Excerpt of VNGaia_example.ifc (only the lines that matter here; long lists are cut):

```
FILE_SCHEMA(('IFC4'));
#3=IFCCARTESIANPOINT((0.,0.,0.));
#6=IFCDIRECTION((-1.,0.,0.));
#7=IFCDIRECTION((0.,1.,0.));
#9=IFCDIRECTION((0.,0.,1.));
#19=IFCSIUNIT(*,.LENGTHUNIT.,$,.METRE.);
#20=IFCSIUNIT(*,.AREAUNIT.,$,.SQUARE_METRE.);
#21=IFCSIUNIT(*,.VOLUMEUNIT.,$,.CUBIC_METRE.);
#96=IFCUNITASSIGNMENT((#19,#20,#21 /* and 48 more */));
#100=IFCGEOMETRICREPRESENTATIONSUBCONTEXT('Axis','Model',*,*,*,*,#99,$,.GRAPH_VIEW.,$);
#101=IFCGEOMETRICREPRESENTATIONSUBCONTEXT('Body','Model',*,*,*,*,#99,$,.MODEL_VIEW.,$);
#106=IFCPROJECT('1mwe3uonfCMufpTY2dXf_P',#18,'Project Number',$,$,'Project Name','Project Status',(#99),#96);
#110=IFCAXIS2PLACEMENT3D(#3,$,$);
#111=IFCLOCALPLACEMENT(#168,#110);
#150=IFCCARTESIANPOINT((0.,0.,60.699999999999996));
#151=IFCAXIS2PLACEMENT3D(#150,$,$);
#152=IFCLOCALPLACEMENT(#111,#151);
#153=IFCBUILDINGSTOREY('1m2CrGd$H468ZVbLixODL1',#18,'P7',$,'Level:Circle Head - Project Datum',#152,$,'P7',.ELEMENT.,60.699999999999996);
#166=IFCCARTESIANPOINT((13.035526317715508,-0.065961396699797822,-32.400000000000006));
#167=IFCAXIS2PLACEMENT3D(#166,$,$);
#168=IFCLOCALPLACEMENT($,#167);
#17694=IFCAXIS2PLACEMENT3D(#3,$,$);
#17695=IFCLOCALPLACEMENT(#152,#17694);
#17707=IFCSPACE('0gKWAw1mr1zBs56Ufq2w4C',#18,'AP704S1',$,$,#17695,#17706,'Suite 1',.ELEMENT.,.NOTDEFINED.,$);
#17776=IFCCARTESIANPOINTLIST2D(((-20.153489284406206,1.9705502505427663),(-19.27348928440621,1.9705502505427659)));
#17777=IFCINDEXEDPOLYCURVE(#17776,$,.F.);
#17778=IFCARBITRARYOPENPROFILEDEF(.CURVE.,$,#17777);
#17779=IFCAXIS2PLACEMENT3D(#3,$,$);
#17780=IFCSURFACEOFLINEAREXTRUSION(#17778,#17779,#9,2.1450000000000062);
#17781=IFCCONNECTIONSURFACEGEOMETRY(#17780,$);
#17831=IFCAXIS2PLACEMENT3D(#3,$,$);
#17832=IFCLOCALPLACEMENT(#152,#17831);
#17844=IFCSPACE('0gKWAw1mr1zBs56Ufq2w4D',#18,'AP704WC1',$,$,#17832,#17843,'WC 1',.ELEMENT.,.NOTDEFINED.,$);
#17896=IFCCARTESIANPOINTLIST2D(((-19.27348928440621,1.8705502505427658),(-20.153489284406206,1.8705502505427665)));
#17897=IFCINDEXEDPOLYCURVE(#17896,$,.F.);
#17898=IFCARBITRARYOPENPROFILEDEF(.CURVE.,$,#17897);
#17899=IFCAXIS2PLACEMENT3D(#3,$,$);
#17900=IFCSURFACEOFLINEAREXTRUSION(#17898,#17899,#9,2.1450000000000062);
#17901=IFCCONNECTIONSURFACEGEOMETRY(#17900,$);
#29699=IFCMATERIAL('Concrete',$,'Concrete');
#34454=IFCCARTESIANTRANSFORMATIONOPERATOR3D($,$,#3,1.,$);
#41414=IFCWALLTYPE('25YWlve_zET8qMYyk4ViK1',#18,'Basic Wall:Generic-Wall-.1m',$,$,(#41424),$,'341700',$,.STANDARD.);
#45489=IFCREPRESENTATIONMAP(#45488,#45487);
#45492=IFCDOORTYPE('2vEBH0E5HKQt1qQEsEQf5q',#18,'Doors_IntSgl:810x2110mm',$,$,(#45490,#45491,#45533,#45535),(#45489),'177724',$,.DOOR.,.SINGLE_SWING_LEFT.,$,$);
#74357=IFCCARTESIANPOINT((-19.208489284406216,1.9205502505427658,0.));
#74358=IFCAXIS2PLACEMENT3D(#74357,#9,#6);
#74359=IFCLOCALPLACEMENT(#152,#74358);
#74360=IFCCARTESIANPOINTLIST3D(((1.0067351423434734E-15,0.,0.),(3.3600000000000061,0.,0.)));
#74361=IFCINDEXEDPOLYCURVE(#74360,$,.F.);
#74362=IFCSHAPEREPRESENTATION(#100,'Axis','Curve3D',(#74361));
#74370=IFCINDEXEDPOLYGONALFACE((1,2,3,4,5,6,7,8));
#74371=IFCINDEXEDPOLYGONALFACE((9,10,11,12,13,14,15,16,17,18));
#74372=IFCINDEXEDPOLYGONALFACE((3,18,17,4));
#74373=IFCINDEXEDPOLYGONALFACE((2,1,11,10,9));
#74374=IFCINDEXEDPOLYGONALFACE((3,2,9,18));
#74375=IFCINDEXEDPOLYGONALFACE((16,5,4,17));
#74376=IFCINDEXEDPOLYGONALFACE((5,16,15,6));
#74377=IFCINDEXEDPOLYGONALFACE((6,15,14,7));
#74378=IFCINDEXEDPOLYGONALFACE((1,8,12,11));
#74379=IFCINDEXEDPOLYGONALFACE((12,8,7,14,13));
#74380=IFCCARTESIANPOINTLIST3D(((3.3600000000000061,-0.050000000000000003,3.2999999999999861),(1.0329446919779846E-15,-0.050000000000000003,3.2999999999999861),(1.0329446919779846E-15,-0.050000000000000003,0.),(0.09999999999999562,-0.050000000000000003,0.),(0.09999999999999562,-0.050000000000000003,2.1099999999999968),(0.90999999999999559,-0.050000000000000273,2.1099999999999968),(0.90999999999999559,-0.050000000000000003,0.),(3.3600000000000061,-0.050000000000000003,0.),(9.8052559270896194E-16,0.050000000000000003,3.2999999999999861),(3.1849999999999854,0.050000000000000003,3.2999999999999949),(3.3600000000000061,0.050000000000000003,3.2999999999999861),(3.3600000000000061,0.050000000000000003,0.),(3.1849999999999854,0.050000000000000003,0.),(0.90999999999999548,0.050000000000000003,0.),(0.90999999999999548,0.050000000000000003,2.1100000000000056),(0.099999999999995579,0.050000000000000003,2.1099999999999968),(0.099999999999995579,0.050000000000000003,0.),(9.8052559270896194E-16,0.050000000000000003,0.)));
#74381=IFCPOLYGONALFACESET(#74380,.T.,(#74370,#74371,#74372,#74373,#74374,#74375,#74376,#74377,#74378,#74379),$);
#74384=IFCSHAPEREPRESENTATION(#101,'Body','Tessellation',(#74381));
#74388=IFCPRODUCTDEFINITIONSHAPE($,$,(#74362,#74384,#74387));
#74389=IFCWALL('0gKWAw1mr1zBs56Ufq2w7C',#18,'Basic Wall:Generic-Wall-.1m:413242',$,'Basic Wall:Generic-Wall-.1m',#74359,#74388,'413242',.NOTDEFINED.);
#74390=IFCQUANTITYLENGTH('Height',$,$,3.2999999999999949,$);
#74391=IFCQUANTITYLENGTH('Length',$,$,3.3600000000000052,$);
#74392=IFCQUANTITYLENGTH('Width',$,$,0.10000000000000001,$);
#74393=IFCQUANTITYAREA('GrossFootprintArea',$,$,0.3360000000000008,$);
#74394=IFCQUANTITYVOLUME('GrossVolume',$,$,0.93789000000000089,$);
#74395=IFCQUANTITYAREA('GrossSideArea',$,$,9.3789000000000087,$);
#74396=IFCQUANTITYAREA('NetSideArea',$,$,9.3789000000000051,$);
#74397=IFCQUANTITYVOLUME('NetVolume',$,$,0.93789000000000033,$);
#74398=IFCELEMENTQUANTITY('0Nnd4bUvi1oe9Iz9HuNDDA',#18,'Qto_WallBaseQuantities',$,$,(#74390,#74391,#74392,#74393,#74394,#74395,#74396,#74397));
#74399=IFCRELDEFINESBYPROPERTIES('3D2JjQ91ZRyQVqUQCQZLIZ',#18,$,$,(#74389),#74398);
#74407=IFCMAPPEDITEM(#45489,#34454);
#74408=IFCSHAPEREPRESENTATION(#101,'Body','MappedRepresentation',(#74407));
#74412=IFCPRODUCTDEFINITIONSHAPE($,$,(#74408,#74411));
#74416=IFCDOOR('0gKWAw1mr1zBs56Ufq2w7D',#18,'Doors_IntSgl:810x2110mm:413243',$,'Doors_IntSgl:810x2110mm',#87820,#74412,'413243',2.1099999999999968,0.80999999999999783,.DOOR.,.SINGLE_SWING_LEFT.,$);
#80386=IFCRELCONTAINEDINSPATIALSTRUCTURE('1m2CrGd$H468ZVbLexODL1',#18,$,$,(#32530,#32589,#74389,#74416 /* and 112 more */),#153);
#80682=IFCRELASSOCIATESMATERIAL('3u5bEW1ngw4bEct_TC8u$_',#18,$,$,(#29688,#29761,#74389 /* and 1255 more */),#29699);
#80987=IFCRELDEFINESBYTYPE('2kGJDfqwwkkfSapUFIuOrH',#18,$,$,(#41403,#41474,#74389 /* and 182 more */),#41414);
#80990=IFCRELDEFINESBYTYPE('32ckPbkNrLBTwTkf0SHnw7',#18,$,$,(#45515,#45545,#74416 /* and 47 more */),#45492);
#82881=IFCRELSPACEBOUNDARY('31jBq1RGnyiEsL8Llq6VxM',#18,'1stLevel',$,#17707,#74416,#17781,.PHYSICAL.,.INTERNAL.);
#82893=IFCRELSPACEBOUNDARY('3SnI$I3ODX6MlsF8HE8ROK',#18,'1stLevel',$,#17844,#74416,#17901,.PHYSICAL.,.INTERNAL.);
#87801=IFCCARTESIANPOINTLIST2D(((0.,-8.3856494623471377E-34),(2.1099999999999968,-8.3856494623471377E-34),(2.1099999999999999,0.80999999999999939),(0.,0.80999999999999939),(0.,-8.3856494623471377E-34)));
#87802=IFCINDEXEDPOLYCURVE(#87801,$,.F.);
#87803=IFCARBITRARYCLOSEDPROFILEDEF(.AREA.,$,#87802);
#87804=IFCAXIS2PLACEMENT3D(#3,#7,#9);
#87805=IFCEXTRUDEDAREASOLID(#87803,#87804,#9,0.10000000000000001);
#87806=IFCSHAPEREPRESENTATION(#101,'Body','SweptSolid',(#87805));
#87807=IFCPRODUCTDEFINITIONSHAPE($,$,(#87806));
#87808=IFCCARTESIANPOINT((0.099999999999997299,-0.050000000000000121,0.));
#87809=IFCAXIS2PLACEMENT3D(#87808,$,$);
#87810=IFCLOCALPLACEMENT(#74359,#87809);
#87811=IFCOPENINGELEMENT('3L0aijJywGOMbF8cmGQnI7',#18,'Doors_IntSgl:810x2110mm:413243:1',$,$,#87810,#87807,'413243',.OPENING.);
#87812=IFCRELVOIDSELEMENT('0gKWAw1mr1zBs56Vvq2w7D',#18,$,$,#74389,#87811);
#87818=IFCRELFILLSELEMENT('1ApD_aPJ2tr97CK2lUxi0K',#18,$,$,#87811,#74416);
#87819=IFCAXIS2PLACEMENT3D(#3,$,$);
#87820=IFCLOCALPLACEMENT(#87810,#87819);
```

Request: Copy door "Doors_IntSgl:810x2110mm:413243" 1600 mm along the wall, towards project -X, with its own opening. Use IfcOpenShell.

```python
import numpy as np
import ifcopenshell
import ifcopenshell.api.feature
import ifcopenshell.api.geometry
import ifcopenshell.api.pset
import ifcopenshell.api.root
import ifcopenshell.geom
import ifcopenshell.util.element
import ifcopenshell.util.placement
import ifcopenshell.util.shape
import ifcopenshell.util.unit

model = ifcopenshell.open("VNGaia_example.ifc")
unit_scale = ifcopenshell.util.unit.calculate_unit_scale(model)
area_scale = ifcopenshell.util.unit.calculate_unit_scale(model, "AREAUNIT")
volume_scale = ifcopenshell.util.unit.calculate_unit_scale(model, "VOLUMEUNIT")
settings = ifcopenshell.geom.settings()


def volume(element):
    """Net volume in cubic metres, openings subtracted."""
    shape = ifcopenshell.geom.create_shape(settings, element)
    return ifcopenshell.util.shape.get_volume(shape.geometry)


def reuse_history(source, copy):
    """copy_class also copies each property set's owner history, people and application; keep the originals."""
    for rel in copy.IsDefinedBy:
        if rel.is_a("IfcRelDefinesByProperties") and (history := rel.RelatingPropertyDefinition.OwnerHistory):
            rel.RelatingPropertyDefinition.OwnerHistory = source.OwnerHistory
            ifcopenshell.util.element.remove_deep2(model, history)


door = model.by_guid("0gKWAw1mr1zBs56Ufq2w7D")
opening = door.FillsVoids[0].RelatingOpeningElement
wall = opening.VoidsElements[0].RelatingBuildingElement
before = volume(wall)
shift = ifcopenshell.util.placement.get_local_placement(wall.ObjectPlacement)[:3, 0] * 1.6 / unit_scale

# copy_class copies the void relationship, type, container and properties, but no geometry.
new_opening = ifcopenshell.api.root.copy_class(model, product=opening)
new_opening.Representation = ifcopenshell.util.element.copy_deep(
    model, opening.Representation, exclude=["IfcGeometricRepresentationContext", "IfcRepresentationMap"]
)
new_opening.Name = "Doors_IntSgl:810x2110mm"
new_opening.Tag = None
reuse_history(opening, new_opening)
new_door = ifcopenshell.api.root.copy_class(model, product=door)
new_door.Representation = ifcopenshell.util.element.copy_deep(
    model, door.Representation, exclude=["IfcGeometricRepresentationContext", "IfcRepresentationMap"]
)
new_door.Name = "Doors_IntSgl:810x2110mm"
new_door.Tag = None
reuse_history(door, new_door)
ifcopenshell.api.feature.add_filling(model, opening=new_opening, element=new_door)

for old, new in ((opening, new_opening), (door, new_door)):
    matrix = ifcopenshell.util.placement.get_local_placement(old.ObjectPlacement)
    matrix[:3, 3] += shift
    ifcopenshell.api.geometry.edit_object_placement(model, product=new, matrix=matrix, is_si=False)

# The copied space boundaries still share their surfaces with the original.
for rel in new_door.ProvidesBoundaries:
    if rel.ConnectionGeometry:
        rel.ConnectionGeometry = ifcopenshell.util.element.copy_deep(model, rel.ConnectionGeometry)

# Space boundary surfaces are stored in each space's coordinates; move them too.
for rel in new_door.ProvidesBoundaries:
    if not rel.ConnectionGeometry:
        continue
    surface = rel.ConnectionGeometry.SurfaceOnRelatingElement
    space_matrix = ifcopenshell.util.placement.get_local_placement(rel.RelatingSpace.ObjectPlacement)
    point = np.array(surface.Position.Location.Coordinates) + space_matrix[:3, :3].T @ shift
    surface.Position = model.createIfcAxis2Placement3D(
        model.createIfcCartesianPoint(point.tolist()), surface.Position.Axis, surface.Position.RefDirection
    )

after = volume(wall)
thickness = 0.1  # wall thickness in metres

# Update the wall's stored quantities.
qto = model.by_id(ifcopenshell.util.element.get_pset(wall, "Qto_WallBaseQuantities", should_inherit=False)["id"])
ifcopenshell.api.pset.edit_qto(model, qto=qto, properties={
    "NetSideArea": after / thickness / area_scale,
    "NetVolume": after / volume_scale,
})

print(f"wall volume {before:.3f} -> {after:.3f} m3")

model.write("VNGaia_example_rev.ifc")
```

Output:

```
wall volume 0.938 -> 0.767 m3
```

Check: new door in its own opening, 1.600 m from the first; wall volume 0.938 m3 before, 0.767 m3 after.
